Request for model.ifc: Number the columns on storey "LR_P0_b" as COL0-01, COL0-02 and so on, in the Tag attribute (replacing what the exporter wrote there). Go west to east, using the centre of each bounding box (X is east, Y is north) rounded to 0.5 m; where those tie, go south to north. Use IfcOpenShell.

First a look at what the model holds.

```python
import ifcopenshell
import ifcopenshell.util.element
import ifcopenshell.util.placement

model = ifcopenshell.open("model.ifc")
print(model.schema)
storey = next(s for s in model.by_type("IfcBuildingStorey") if s.Name == "LR_P0_b")
columns = [e for e in ifcopenshell.util.element.get_decomposition(storey) if e.is_a("IfcColumn")]
for e in sorted(columns, key=lambda e: e.id()):
    origin = ifcopenshell.util.placement.get_local_placement(e.ObjectPlacement)[:3, 3]
    print(e.id(), e.Tag, e.Name, origin.round(2) + 0.0, sep=" | ")
```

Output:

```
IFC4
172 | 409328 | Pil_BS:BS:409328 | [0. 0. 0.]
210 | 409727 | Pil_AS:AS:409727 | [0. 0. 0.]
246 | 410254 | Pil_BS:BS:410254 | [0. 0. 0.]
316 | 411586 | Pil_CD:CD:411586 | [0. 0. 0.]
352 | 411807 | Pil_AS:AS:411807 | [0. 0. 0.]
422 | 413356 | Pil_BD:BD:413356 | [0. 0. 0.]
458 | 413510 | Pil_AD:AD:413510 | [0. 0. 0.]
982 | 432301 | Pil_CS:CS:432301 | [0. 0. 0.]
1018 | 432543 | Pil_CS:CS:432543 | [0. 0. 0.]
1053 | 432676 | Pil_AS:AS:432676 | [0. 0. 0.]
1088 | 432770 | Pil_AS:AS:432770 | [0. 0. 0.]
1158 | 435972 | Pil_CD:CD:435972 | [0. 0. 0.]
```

```python
import ifcopenshell
import ifcopenshell.geom
import ifcopenshell.util.element
import ifcopenshell.util.shape

model = ifcopenshell.open("model.ifc")
settings = ifcopenshell.geom.settings()
settings.set("use-world-coords", True)


def centre(element):
    shape = ifcopenshell.geom.create_shape(settings, element)
    return ifcopenshell.util.shape.get_bbox_centroid(shape.geometry)


storey = next(s for s in model.by_type("IfcBuildingStorey") if s.Name == "LR_P0_b")
columns = [e for e in ifcopenshell.util.element.get_decomposition(storey) if e.is_a("IfcColumn")]

# Insertion points can sit at a corner or the storey origin, so sort by the geometry (in metres).
centres = {e: centre(e) for e in columns}
columns.sort(key=lambda e: (round(centres[e][0] / 0.5), centres[e][1]))

for i, e in enumerate(columns, start=1):
    number = f"COL0-{i:02d}"
    e.Tag = number
    print(e.id(), number)

model.write("model_v2.ifc")
```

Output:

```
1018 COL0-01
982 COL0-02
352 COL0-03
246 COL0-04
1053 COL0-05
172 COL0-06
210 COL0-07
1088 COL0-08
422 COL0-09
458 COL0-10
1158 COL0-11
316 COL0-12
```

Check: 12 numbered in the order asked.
